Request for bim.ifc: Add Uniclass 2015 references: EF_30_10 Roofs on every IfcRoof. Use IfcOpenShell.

First a look at what the model holds.

```python
import ifcopenshell

model = ifcopenshell.open("bim.ifc")
print(model.schema)
print("classifications:", [c.Name for c in model.by_type("IfcClassification")])
for ifc_class in ("IfcDoor", "IfcRoof", "IfcStair", "IfcWall", "IfcWindow"):
    print(ifc_class, len(model.by_type(ifc_class)))
```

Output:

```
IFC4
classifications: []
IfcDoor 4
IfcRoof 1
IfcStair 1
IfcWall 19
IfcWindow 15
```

```python
import ifcopenshell
import ifcopenshell.api.classification

model = ifcopenshell.open("bim.ifc")

system = ifcopenshell.api.classification.add_classification(model, classification="Uniclass 2015")

codes = {
    "IfcRoof": ("EF_30_10", "Roofs"),
}
for ifc_class, (code, name) in codes.items():
    products = model.by_type(ifc_class)
    ifcopenshell.api.classification.add_reference(
        model, products=products, classification=system, identification=code, name=name
    )
    print(code, len(products))

model.write("bim-out.ifc")
```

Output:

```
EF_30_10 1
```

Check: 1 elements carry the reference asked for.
